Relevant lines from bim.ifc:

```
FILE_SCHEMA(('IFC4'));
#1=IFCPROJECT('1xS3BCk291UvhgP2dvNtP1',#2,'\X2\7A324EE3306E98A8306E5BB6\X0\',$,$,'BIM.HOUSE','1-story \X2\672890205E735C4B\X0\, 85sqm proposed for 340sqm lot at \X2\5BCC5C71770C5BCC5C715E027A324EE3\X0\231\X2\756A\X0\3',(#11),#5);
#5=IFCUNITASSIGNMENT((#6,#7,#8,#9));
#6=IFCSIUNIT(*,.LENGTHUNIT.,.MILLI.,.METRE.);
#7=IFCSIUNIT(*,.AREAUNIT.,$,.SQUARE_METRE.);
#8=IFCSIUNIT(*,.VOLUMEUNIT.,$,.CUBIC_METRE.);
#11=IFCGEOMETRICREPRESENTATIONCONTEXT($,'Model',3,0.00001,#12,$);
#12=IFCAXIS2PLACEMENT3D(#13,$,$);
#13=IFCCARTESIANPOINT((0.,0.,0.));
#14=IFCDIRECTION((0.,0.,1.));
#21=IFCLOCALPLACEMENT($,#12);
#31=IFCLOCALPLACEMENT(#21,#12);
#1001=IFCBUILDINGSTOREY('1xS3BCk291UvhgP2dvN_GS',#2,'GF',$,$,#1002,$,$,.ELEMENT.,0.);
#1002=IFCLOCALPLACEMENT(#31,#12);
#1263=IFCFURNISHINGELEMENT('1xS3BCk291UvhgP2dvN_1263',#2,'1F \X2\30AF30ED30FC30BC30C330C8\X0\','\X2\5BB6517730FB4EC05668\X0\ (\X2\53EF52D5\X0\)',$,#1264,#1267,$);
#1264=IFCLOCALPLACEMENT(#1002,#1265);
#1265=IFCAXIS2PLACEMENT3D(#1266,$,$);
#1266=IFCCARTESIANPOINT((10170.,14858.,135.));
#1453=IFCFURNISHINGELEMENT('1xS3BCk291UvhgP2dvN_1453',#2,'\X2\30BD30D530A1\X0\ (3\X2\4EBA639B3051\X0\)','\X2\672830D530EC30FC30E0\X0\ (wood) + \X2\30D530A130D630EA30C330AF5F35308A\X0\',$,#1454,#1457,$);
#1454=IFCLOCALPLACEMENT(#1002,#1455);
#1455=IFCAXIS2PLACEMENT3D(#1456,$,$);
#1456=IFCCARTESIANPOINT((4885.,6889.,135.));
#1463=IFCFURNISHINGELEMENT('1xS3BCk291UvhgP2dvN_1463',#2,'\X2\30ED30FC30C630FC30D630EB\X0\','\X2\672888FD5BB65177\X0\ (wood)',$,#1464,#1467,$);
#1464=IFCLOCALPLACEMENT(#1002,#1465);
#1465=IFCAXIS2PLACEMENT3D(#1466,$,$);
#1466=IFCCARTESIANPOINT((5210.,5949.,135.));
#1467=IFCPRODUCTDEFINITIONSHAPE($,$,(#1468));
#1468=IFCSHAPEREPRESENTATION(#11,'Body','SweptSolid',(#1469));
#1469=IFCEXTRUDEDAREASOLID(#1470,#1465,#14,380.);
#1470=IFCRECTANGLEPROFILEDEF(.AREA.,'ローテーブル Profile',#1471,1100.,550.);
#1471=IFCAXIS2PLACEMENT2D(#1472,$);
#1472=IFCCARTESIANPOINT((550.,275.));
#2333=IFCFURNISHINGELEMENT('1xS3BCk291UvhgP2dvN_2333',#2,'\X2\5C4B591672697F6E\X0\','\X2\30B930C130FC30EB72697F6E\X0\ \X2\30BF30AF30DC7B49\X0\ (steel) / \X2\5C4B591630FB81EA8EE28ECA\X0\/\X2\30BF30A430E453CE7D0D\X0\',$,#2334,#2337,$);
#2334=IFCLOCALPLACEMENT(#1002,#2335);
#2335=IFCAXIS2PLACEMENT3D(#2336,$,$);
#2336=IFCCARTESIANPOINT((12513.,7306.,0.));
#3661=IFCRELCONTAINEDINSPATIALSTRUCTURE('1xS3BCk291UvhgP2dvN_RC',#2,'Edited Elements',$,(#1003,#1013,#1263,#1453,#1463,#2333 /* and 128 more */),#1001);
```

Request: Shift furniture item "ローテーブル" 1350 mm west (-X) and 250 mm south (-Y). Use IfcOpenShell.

```python
import ifcopenshell
import ifcopenshell.api.geometry
import ifcopenshell.util.placement

model = ifcopenshell.open("bim.ifc")

item = model.by_guid("1xS3BCk291UvhgP2dvN_1463")
matrix = ifcopenshell.util.placement.get_local_placement(item.ObjectPlacement)
matrix[0, 3] -= 1350.0
matrix[1, 3] -= 250.0
ifcopenshell.api.geometry.edit_object_placement(model, product=item, matrix=matrix, is_si=False)

print(ifcopenshell.util.placement.get_local_placement(item.ObjectPlacement).round(3) + 0.0)

model.write("bim-out.ifc")
```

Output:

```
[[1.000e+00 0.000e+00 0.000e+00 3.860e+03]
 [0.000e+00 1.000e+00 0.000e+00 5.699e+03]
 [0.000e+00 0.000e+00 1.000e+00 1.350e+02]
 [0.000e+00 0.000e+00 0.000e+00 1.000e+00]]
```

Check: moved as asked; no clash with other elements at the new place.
